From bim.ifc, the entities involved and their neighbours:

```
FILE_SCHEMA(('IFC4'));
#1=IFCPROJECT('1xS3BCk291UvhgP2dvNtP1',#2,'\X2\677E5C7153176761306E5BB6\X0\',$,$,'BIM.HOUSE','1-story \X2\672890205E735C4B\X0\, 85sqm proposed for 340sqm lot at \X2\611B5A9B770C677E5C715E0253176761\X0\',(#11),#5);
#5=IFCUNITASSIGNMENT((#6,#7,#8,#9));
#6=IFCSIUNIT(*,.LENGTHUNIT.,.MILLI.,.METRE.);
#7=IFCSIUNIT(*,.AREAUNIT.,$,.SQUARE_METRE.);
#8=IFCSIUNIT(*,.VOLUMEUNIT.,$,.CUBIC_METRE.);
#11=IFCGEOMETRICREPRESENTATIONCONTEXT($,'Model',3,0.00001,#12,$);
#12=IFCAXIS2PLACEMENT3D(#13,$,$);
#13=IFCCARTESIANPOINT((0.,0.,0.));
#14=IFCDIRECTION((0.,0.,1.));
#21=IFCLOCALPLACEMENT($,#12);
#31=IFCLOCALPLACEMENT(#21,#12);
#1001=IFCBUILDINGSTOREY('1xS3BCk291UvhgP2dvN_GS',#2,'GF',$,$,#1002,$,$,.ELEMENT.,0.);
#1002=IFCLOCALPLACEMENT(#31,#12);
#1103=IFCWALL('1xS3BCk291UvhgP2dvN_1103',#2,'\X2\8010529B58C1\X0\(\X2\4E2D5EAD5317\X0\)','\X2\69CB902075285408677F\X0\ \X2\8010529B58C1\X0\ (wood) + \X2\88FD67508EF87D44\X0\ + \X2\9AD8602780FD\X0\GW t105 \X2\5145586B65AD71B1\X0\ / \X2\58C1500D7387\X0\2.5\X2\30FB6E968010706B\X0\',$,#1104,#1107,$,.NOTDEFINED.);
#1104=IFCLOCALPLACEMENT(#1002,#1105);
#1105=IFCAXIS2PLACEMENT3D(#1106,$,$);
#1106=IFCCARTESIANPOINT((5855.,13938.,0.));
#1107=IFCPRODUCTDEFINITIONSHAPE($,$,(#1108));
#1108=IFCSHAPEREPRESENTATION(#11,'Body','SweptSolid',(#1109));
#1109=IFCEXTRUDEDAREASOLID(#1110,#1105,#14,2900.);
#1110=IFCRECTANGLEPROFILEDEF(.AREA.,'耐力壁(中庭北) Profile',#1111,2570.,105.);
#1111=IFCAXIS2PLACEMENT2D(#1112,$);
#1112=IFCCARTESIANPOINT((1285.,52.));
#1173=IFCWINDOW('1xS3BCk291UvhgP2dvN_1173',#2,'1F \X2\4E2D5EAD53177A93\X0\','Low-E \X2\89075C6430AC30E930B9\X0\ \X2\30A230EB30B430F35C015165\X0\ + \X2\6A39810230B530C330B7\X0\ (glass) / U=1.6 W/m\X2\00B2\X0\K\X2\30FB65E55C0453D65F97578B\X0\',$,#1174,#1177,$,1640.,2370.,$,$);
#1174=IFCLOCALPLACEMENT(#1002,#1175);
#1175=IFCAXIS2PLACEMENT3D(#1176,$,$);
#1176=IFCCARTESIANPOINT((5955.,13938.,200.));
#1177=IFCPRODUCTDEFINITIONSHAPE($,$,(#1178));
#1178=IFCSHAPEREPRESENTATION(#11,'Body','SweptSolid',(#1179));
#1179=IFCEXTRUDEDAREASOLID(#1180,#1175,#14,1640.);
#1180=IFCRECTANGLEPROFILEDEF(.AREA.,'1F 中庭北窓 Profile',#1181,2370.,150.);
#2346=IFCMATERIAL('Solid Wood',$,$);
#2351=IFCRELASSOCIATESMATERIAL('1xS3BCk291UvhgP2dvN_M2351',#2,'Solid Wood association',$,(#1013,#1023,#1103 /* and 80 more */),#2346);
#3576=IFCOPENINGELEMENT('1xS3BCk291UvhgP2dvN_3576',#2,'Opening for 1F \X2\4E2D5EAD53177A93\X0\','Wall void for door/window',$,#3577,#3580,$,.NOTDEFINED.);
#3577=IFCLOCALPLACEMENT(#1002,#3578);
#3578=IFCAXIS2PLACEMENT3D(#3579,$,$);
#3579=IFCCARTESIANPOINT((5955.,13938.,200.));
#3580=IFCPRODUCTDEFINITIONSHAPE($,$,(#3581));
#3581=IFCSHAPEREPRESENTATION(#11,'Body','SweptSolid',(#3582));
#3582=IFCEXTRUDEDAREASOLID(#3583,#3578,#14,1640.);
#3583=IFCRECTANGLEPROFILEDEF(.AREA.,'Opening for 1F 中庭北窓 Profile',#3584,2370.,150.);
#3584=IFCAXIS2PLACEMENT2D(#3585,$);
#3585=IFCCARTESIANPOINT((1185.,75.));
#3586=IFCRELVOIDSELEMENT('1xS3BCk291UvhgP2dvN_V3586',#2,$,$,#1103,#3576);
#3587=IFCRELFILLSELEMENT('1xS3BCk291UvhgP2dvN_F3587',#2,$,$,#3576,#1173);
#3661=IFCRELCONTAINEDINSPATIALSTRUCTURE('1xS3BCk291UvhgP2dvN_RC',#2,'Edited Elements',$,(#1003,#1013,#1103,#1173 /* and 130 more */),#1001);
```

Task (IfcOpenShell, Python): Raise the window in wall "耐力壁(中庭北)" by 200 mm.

```python
import numpy as np
import ifcopenshell
import ifcopenshell.api.geometry
import ifcopenshell.util.placement
import ifcopenshell.util.unit

model = ifcopenshell.open("bim.ifc")
unit_scale = ifcopenshell.util.unit.calculate_unit_scale(model)

window = model.by_id(1173)
opening = window.FillsVoids[0].RelatingOpeningElement
dz = 0.2 / unit_scale

shift = np.array([0.0, 0.0, dz])
# The window is not placed relative to its opening, so move both.
for product in (opening, window):
    matrix = ifcopenshell.util.placement.get_local_placement(product.ObjectPlacement)
    matrix[:3, 3] += shift
    ifcopenshell.api.geometry.edit_object_placement(model, product=product, matrix=matrix, is_si=False)

print(f"moved by {dz * unit_scale:+.3f} m")

model.write("bim_edited.ifc")
```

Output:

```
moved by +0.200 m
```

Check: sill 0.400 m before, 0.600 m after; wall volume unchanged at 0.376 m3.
